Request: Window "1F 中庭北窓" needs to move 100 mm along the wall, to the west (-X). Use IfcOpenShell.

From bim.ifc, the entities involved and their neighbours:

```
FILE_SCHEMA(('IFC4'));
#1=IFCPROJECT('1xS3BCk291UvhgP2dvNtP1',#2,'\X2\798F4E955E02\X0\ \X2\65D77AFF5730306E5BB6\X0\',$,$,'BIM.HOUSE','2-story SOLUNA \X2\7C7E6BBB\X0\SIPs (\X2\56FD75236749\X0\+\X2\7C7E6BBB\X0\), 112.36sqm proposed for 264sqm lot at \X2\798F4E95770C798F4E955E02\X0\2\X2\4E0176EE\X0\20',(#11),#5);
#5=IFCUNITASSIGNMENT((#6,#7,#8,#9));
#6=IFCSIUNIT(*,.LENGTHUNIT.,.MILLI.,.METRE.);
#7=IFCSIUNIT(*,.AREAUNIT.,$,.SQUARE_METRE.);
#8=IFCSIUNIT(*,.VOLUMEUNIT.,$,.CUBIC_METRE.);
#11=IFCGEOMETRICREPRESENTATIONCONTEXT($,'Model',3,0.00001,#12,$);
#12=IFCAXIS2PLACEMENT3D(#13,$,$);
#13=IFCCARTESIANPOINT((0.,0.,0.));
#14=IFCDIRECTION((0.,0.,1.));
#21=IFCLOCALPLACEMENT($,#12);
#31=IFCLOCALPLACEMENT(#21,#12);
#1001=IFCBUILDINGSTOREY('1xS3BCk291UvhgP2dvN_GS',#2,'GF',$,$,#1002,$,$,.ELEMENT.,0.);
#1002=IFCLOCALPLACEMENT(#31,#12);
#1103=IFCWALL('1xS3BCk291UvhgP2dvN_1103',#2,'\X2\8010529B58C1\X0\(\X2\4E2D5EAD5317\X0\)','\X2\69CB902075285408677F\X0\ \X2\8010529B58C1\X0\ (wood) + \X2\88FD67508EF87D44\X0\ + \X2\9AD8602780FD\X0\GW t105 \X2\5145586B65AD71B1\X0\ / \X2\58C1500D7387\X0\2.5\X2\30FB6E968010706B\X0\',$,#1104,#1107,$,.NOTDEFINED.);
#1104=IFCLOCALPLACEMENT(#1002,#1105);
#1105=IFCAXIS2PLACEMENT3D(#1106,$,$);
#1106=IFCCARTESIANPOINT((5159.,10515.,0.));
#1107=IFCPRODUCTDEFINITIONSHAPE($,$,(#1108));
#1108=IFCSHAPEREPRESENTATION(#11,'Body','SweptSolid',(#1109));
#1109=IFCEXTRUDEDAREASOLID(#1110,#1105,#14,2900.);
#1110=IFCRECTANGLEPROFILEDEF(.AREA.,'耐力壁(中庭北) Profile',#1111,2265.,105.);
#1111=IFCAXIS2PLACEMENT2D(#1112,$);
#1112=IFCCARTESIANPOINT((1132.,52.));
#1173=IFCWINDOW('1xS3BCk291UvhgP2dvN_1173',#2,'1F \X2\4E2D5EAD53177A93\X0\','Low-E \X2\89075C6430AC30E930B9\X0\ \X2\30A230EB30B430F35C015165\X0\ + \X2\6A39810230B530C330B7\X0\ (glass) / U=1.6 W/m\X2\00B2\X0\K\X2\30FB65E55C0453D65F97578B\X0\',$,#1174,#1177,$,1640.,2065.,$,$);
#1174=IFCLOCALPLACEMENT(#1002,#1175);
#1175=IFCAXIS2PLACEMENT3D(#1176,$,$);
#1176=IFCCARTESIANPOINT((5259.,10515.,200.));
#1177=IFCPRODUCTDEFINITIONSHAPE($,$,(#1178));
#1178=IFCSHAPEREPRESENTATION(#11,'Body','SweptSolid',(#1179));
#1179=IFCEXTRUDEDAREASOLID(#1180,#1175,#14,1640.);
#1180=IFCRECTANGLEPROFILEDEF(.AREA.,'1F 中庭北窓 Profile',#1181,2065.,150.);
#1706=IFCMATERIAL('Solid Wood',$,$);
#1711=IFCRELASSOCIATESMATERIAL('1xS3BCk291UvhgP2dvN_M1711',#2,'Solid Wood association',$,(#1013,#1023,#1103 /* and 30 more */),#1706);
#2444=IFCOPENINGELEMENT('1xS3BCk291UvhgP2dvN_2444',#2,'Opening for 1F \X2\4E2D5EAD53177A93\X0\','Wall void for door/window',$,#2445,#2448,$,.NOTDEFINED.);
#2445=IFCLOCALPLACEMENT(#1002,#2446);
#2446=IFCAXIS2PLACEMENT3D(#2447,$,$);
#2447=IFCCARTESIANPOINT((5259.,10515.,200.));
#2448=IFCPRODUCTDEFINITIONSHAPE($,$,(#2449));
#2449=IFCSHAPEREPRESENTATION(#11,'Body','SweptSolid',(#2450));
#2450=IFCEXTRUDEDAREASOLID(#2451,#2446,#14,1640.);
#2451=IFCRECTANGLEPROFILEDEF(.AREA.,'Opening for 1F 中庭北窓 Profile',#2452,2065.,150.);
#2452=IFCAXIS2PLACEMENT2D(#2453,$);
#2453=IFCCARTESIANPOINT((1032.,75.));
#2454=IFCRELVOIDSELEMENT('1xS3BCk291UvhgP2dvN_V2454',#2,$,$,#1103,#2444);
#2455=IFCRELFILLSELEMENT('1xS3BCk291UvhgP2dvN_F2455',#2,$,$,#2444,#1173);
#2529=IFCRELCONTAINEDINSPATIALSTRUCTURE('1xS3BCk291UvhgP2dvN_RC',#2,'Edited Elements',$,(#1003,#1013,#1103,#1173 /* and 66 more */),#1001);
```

```python
import ifcopenshell
import ifcopenshell.api.geometry
import ifcopenshell.util.placement

model = ifcopenshell.open("bim.ifc")

window = model.by_guid("1xS3BCk291UvhgP2dvN_1173")
opening = window.FillsVoids[0].RelatingOpeningElement
wall = opening.VoidsElements[0].RelatingBuildingElement

wall_matrix = ifcopenshell.util.placement.get_local_placement(wall.ObjectPlacement)
shift = wall_matrix[:3, 0] * -100.0
before = ifcopenshell.util.placement.get_local_placement(window.ObjectPlacement)[:3, 3].copy()

# The window is not placed relative to its opening, so move both.
for product in (opening, window):
    matrix = ifcopenshell.util.placement.get_local_placement(product.ObjectPlacement)
    matrix[:3, 3] += shift
    ifcopenshell.api.geometry.edit_object_placement(model, product=product, matrix=matrix, is_si=False)

after = ifcopenshell.util.placement.get_local_placement(window.ObjectPlacement)[:3, 3]
print("window moved by", (after - before).round(3) + 0.0)

model.write("bim_rev.ifc")
```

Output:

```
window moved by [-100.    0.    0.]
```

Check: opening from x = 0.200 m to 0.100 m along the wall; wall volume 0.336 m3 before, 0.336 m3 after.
